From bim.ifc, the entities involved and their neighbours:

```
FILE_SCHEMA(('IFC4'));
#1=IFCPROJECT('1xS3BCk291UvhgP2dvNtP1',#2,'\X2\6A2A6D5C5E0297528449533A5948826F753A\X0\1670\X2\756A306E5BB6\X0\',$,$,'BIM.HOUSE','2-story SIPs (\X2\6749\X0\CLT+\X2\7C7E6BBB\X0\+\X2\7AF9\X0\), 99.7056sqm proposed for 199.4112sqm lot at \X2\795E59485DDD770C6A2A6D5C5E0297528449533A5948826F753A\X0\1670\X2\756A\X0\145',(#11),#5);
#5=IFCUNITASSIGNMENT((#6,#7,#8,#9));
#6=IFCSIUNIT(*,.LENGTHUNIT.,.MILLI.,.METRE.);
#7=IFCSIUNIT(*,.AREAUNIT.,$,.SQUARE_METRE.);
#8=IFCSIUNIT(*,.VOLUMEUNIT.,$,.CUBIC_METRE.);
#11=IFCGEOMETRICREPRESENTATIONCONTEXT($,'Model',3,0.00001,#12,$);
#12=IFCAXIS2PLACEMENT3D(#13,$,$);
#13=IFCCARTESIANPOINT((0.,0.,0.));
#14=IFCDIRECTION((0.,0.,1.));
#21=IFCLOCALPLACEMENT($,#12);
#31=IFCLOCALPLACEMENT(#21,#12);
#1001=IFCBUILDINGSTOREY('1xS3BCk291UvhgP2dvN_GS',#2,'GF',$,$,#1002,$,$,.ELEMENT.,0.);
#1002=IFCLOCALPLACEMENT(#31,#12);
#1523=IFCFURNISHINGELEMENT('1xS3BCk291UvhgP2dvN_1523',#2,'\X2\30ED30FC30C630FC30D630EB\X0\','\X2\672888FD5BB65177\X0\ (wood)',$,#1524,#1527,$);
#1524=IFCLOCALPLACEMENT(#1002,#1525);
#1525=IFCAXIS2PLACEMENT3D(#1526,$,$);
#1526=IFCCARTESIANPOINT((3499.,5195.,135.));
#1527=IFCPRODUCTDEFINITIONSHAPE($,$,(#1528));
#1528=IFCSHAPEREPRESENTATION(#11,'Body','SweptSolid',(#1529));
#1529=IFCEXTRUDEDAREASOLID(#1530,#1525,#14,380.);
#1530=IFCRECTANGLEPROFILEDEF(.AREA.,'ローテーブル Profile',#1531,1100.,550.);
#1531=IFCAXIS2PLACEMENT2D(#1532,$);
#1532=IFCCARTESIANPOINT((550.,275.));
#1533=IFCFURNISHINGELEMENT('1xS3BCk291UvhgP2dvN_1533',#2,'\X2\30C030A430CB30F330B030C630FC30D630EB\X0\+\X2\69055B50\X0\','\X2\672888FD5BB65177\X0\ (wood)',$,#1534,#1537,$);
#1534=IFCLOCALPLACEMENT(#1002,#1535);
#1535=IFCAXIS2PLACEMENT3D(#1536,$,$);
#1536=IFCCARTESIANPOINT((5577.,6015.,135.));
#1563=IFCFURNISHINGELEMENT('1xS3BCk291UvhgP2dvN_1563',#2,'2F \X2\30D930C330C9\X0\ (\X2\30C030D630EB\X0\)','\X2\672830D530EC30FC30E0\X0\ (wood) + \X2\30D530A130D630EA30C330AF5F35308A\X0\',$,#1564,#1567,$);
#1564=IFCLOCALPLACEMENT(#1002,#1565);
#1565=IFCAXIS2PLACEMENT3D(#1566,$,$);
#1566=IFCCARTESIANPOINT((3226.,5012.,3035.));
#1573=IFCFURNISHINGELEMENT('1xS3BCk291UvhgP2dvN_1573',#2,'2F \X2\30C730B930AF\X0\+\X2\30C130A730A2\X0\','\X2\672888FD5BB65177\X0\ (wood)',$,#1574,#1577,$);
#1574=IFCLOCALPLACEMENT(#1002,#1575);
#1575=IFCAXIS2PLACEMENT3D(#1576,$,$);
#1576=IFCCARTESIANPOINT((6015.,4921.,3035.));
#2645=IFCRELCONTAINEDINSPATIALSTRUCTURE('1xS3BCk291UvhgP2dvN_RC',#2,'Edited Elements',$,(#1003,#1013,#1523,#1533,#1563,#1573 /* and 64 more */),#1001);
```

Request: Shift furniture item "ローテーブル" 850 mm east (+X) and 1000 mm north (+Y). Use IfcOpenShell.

```python
import ifcopenshell
import ifcopenshell.api.geometry
import ifcopenshell.util.placement

model = ifcopenshell.open("bim.ifc")

item = model.by_guid("1xS3BCk291UvhgP2dvN_1523")
matrix = ifcopenshell.util.placement.get_local_placement(item.ObjectPlacement)
matrix[0, 3] += 850.0
matrix[1, 3] += 1000.0
ifcopenshell.api.geometry.edit_object_placement(model, product=item, matrix=matrix, is_si=False)

print(ifcopenshell.util.placement.get_local_placement(item.ObjectPlacement).round(3) + 0.0)

model.write("bim_v2.ifc")
```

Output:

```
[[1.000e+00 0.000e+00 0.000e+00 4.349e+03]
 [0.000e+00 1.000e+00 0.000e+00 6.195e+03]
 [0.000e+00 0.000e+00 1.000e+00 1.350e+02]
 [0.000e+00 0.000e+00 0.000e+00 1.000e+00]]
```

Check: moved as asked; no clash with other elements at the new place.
